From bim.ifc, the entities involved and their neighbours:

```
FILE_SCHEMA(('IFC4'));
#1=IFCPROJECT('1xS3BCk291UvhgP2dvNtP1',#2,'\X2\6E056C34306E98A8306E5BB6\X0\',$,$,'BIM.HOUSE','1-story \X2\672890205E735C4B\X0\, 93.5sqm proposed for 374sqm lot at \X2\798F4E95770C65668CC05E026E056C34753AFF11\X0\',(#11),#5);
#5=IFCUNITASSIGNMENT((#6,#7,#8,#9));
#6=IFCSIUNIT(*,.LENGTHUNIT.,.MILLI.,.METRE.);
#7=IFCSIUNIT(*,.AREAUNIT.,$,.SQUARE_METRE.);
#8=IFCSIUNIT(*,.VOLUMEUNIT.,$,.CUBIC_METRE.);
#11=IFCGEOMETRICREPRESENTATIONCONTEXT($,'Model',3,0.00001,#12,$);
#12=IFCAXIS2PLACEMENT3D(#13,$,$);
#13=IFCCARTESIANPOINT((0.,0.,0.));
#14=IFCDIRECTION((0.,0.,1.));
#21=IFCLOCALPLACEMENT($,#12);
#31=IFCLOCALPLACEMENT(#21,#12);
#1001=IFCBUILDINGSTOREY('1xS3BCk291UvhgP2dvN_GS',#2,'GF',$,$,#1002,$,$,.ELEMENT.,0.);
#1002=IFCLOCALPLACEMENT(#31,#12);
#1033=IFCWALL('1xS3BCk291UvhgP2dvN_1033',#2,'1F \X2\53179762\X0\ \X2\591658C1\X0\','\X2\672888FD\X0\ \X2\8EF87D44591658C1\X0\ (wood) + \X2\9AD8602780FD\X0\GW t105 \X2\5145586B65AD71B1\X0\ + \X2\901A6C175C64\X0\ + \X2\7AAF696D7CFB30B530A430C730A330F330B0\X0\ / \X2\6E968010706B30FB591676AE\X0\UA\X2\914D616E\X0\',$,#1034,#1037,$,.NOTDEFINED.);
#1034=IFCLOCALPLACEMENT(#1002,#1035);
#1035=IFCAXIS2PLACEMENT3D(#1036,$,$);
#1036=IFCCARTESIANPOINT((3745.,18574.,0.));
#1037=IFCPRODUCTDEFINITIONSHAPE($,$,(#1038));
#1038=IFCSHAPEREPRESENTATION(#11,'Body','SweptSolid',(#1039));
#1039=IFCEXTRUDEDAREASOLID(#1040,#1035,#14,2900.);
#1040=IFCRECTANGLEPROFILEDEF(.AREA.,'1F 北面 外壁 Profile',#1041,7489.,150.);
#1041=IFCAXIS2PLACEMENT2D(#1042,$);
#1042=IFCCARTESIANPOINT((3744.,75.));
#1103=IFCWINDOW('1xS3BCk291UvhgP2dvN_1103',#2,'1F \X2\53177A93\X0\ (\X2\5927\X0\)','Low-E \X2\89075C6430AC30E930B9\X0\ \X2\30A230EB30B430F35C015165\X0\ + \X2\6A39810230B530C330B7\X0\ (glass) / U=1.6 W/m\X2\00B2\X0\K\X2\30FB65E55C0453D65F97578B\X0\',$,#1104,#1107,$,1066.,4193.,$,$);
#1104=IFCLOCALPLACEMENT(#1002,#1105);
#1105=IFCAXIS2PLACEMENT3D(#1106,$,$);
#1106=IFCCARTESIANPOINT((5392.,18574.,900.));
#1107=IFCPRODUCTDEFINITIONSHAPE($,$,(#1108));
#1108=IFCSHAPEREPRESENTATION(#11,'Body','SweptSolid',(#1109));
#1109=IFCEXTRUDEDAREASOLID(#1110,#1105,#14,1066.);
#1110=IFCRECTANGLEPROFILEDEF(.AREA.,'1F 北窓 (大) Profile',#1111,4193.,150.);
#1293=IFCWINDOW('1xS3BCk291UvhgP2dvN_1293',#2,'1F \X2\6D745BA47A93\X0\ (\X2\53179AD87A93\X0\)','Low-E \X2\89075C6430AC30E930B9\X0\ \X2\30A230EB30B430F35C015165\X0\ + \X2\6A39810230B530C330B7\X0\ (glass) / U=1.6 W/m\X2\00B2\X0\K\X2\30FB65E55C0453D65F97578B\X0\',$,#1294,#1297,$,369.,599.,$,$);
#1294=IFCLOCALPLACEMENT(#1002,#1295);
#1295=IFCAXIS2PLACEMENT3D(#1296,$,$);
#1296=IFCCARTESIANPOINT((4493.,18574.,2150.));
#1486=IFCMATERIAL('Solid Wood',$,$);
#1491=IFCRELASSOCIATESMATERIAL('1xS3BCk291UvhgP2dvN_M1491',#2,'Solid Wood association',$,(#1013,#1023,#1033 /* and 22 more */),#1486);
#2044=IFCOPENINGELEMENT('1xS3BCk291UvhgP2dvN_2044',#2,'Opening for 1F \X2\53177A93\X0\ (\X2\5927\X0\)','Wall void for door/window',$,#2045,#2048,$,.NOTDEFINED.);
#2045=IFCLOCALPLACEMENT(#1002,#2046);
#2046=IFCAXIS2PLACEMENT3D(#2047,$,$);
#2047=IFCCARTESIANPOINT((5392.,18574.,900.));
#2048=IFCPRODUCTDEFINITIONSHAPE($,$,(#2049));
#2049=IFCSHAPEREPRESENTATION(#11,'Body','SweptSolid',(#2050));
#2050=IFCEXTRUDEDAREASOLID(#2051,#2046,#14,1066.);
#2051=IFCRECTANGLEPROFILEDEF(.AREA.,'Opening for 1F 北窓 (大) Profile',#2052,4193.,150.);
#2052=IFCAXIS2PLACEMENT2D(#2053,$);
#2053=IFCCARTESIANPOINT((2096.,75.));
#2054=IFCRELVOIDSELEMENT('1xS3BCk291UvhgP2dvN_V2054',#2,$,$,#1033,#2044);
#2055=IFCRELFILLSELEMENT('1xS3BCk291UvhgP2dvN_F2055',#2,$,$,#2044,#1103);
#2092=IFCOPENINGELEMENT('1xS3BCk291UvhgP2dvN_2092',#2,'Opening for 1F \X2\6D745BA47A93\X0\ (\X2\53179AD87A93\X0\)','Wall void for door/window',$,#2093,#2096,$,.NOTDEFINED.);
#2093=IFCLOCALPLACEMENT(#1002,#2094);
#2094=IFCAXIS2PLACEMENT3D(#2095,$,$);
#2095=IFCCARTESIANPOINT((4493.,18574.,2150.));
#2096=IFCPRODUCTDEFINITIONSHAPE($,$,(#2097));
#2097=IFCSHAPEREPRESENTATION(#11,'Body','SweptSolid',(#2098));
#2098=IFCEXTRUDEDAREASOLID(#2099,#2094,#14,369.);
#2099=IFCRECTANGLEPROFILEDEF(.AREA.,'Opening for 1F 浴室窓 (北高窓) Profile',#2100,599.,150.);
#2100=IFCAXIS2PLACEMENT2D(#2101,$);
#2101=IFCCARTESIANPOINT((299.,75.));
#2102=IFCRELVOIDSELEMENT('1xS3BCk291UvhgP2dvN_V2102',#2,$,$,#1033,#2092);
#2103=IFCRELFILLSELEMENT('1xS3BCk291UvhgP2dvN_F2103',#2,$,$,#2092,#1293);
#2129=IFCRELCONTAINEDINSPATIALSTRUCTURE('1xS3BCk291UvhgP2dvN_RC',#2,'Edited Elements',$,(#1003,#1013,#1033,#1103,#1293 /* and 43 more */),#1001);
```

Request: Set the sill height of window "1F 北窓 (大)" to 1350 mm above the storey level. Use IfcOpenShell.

```python
import numpy as np
import ifcopenshell
import ifcopenshell.api.geometry
import ifcopenshell.geom
import ifcopenshell.util.element
import ifcopenshell.util.placement
import ifcopenshell.util.shape
import ifcopenshell.util.unit

model = ifcopenshell.open("bim.ifc")
unit_scale = ifcopenshell.util.unit.calculate_unit_scale(model)

window = model.by_guid("1xS3BCk291UvhgP2dvN_1103")
opening = window.FillsVoids[0].RelatingOpeningElement
storey = ifcopenshell.util.element.get_container(window, ifc_class="IfcBuildingStorey")
level = ifcopenshell.util.placement.get_local_placement(storey.ObjectPlacement)[2, 3]

# The opening's origin need not be at the sill, so measure its lowest point.
shape = ifcopenshell.geom.create_shape(ifcopenshell.geom.settings(), opening)
bottom = ifcopenshell.util.shape.get_shape_bottom_elevation(shape, shape.geometry) / unit_scale
dz = level + 1350.0 - bottom

shift = np.array([0.0, 0.0, dz])
# The window is not placed relative to its opening, so move both.
for product in (opening, window):
    matrix = ifcopenshell.util.placement.get_local_placement(product.ObjectPlacement)
    matrix[:3, 3] += shift
    ifcopenshell.api.geometry.edit_object_placement(model, product=product, matrix=matrix, is_si=False)

print(f"moved by {dz * unit_scale:+.3f} m")

model.write("bim-out.ifc")
```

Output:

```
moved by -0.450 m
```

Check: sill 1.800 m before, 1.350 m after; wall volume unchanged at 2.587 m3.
